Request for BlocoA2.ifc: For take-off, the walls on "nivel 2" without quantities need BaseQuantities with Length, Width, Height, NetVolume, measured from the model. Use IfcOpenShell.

First a look at what the model holds.

```python
import ifcopenshell
import ifcopenshell.util.element
import ifcopenshell.util.unit

model = ifcopenshell.open("BlocoA2.ifc")
print(model.schema)
for unit_type in ("LENGTHUNIT", "AREAUNIT", "VOLUMEUNIT"):
    print(unit_type, ifcopenshell.util.unit.calculate_unit_scale(model, unit_type))
storey = next(s for s in model.by_type("IfcBuildingStorey") if s.Name == "nivel 2")
walls = [e for e in ifcopenshell.util.element.get_decomposition(storey) if e.is_a("IfcWall")]
for e in sorted(walls, key=lambda e: e.id()):
    print(e.id(), e.is_a(), e.Name, list(ifcopenshell.util.element.get_psets(e, qtos_only=True)), sep=" | ")
```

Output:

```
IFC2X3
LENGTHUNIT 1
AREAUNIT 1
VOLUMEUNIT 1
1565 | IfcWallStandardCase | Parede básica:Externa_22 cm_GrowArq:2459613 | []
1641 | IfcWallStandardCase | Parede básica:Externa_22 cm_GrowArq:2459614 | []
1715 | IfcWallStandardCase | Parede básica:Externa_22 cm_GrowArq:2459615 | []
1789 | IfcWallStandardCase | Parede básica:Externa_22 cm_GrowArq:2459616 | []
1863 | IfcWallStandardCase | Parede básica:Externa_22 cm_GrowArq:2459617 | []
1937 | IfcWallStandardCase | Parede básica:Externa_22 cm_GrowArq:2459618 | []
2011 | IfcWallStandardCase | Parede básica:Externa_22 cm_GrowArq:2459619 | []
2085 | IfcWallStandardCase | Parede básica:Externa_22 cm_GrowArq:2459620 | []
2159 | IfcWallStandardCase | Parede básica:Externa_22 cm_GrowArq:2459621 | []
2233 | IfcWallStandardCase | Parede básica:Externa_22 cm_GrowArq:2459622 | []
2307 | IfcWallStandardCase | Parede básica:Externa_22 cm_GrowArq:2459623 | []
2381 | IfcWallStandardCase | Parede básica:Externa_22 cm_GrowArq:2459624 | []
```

```python
import ifcopenshell
import ifcopenshell.api.pset
import ifcopenshell.geom
import ifcopenshell.util.element
import ifcopenshell.util.shape
import ifcopenshell.util.unit

model = ifcopenshell.open("BlocoA2.ifc")
unit_scale = ifcopenshell.util.unit.calculate_unit_scale(model)
volume_scale = ifcopenshell.util.unit.calculate_unit_scale(model, "VOLUMEUNIT")
settings = ifcopenshell.geom.settings()

storey = next(s for s in model.by_type("IfcBuildingStorey") if s.Name == "nivel 2")
walls = [e for e in ifcopenshell.util.element.get_decomposition(storey) if e.is_a("IfcWall")]

for e in sorted(walls, key=lambda e: e.id()):
    if ifcopenshell.util.element.get_psets(e, qtos_only=True, should_inherit=False):
        continue
    # Geometry comes back in metres, in the element's own axes.
    shape = ifcopenshell.geom.create_shape(settings, e)
    values = {
        "Length": ifcopenshell.util.shape.get_x(shape.geometry) / unit_scale,
        "Width": ifcopenshell.util.shape.get_y(shape.geometry) / unit_scale,
        "Height": ifcopenshell.util.shape.get_z(shape.geometry) / unit_scale,
        "NetVolume": ifcopenshell.util.shape.get_volume(shape.geometry) / volume_scale,
    }
    qto = ifcopenshell.api.pset.add_qto(model, product=e, name="BaseQuantities")
    ifcopenshell.api.pset.edit_qto(model, qto=qto, properties=values)
    print(e.id(), {k: round(v, 3) for k, v in values.items()})

model.write("BlocoA2_edited.ifc")
```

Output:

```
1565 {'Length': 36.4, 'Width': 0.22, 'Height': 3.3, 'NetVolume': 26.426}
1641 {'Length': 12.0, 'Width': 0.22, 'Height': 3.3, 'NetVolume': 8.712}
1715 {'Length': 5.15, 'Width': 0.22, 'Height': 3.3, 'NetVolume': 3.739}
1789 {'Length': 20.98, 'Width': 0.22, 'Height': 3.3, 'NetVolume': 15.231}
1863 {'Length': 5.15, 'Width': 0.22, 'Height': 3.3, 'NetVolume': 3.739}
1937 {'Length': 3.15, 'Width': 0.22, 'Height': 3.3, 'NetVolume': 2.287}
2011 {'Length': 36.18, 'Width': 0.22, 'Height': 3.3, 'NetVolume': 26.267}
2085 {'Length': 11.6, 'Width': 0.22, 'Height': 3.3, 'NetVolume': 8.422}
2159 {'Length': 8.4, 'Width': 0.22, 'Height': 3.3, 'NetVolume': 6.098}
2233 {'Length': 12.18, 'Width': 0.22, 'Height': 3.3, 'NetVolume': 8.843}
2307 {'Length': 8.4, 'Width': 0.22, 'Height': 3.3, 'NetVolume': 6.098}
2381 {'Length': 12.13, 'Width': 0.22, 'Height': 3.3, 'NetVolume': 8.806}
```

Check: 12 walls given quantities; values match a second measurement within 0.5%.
